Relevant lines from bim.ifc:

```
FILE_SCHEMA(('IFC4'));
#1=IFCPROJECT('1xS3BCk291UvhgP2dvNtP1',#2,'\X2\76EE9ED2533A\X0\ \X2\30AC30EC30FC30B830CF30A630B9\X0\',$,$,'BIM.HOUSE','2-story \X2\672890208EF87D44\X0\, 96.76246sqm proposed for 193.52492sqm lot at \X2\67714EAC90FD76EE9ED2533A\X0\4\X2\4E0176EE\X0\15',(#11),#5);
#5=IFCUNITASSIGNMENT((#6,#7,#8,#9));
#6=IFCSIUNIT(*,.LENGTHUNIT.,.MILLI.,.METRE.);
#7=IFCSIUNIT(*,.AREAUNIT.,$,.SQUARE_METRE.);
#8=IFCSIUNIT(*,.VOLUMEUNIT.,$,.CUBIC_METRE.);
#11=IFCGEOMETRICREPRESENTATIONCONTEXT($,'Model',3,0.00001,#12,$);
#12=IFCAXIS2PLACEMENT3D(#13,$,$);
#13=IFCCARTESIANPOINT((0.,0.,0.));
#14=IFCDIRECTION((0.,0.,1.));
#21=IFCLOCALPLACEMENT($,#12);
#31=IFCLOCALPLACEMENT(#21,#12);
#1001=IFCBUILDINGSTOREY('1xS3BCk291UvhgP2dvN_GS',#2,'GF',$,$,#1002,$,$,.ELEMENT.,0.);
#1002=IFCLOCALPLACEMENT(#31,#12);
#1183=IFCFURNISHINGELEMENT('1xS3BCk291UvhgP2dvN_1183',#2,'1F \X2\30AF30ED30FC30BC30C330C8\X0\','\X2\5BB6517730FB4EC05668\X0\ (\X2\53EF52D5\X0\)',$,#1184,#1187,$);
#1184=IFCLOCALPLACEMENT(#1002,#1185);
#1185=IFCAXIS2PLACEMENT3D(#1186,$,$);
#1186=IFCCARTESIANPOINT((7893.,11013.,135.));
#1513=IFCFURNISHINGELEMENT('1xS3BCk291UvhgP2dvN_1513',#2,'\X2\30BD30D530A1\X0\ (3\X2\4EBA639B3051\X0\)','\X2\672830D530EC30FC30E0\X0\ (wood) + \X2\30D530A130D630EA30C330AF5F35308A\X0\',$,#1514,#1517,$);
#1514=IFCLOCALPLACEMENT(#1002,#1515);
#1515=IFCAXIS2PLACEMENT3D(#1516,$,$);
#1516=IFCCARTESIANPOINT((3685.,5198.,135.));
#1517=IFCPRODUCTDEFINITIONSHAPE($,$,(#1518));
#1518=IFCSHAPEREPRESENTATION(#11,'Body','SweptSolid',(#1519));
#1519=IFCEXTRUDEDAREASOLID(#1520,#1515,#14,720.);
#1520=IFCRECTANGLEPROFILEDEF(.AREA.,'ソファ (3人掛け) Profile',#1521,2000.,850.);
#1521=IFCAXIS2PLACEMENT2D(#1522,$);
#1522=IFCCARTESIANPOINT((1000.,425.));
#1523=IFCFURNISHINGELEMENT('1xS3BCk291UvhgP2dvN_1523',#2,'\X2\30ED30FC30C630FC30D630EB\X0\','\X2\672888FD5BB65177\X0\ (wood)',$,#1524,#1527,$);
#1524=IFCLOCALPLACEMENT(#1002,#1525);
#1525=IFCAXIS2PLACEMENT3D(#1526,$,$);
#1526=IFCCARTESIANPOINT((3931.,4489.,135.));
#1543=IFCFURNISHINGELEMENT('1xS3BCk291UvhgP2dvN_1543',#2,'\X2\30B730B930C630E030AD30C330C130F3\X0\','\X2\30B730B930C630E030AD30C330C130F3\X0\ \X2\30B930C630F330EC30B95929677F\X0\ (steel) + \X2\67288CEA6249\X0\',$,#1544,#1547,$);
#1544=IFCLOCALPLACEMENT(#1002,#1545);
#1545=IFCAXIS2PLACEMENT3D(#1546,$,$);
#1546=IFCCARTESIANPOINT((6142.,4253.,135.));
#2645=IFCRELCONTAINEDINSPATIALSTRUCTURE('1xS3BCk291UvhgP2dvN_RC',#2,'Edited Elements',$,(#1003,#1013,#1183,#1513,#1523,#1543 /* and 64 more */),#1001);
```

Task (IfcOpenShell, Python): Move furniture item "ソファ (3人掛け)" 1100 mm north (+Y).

```python
import ifcopenshell
import ifcopenshell.api.geometry
import ifcopenshell.util.placement
import ifcopenshell.util.unit

model = ifcopenshell.open("bim.ifc")
unit_scale = ifcopenshell.util.unit.calculate_unit_scale(model)

item = model.by_guid("1xS3BCk291UvhgP2dvN_1513")
matrix = ifcopenshell.util.placement.get_local_placement(item.ObjectPlacement)
matrix[1, 3] += 1.1 / unit_scale
ifcopenshell.api.geometry.edit_object_placement(model, product=item, matrix=matrix, is_si=False)

print(ifcopenshell.util.placement.get_local_placement(item.ObjectPlacement).round(3) + 0.0)

model.write("bim_edited.ifc")
```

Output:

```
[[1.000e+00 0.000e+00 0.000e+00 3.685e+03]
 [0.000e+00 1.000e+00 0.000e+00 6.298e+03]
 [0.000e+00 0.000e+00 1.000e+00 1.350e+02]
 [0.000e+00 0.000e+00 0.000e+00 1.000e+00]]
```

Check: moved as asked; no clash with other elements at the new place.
